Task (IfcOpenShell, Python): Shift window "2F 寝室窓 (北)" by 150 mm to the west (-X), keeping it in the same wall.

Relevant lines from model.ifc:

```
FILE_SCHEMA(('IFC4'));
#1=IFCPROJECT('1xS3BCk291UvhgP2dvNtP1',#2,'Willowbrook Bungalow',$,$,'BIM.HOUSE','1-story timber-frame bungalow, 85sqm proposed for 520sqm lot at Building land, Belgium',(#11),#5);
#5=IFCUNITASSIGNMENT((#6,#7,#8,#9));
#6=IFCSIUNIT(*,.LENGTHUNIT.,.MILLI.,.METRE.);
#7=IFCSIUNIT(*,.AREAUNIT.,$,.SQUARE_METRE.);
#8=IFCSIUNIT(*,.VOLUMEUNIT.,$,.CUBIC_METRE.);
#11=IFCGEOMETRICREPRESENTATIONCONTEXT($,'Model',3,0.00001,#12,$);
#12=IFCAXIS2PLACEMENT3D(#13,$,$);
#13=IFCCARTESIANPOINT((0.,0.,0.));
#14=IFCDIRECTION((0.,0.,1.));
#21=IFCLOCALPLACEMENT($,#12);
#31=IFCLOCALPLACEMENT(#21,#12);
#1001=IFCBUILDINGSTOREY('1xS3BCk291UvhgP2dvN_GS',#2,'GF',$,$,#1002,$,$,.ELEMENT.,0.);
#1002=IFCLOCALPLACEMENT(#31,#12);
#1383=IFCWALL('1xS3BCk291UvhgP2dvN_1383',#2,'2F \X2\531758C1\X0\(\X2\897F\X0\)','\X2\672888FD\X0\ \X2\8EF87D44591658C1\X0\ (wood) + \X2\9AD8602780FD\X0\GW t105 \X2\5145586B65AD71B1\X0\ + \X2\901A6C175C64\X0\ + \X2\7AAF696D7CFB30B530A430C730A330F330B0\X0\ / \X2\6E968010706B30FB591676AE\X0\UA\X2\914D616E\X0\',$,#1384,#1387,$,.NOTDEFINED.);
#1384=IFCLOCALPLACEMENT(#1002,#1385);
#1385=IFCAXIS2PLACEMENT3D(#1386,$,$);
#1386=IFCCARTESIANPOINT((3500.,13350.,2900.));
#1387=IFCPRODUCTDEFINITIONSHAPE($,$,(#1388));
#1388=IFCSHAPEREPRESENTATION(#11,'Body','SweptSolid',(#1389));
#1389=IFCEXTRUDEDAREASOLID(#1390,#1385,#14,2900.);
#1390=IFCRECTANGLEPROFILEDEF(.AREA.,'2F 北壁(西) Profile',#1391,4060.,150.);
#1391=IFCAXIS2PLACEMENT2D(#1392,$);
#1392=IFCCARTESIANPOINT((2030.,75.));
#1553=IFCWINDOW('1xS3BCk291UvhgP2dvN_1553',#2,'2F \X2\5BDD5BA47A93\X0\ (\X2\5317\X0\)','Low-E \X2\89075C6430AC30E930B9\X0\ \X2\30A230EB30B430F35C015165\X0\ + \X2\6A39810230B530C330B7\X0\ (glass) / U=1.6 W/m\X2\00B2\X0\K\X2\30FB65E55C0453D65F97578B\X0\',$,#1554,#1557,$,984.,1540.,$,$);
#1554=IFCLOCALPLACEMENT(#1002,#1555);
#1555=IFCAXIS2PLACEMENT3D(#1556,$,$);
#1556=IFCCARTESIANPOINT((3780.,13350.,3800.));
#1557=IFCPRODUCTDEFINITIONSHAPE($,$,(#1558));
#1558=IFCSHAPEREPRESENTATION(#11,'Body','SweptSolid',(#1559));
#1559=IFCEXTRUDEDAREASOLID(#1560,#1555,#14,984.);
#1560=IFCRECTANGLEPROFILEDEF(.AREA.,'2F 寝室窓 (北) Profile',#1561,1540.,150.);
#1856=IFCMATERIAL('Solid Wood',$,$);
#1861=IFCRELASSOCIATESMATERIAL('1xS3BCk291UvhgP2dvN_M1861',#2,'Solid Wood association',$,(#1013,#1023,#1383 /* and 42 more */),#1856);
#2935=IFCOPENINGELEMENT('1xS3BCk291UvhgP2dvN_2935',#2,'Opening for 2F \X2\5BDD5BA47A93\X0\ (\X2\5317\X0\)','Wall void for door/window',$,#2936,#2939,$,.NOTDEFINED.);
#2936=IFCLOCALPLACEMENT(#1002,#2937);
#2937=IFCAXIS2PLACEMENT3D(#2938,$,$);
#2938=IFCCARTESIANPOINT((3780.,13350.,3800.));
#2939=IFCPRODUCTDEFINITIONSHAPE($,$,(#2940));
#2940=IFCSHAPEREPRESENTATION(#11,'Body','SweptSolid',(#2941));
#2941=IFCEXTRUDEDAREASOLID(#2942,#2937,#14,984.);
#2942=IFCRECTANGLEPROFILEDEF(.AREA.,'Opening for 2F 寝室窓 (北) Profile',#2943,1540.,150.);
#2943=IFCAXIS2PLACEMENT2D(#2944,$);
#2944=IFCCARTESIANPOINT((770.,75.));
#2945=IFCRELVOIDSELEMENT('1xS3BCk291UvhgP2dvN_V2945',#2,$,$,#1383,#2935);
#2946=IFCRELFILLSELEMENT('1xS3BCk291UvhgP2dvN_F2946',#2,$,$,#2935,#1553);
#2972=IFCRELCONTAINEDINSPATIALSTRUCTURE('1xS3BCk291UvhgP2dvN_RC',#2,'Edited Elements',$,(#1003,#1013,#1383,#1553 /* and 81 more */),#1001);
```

```python
import ifcopenshell
import ifcopenshell.api.geometry
import ifcopenshell.util.placement
import ifcopenshell.util.unit

model = ifcopenshell.open("model.ifc")
unit_scale = ifcopenshell.util.unit.calculate_unit_scale(model)

window = model.by_guid("1xS3BCk291UvhgP2dvN_1553")
opening = window.FillsVoids[0].RelatingOpeningElement
wall = opening.VoidsElements[0].RelatingBuildingElement

wall_matrix = ifcopenshell.util.placement.get_local_placement(wall.ObjectPlacement)
shift = wall_matrix[:3, 0] * -0.15 / unit_scale
before = ifcopenshell.util.placement.get_local_placement(window.ObjectPlacement)[:3, 3].copy()

# The window is not placed relative to its opening, so move both.
for product in (opening, window):
    matrix = ifcopenshell.util.placement.get_local_placement(product.ObjectPlacement)
    matrix[:3, 3] += shift
    ifcopenshell.api.geometry.edit_object_placement(model, product=product, matrix=matrix, is_si=False)

after = ifcopenshell.util.placement.get_local_placement(window.ObjectPlacement)[:3, 3]
print("window moved by", (after - before).round(3) + 0.0)

model.write("model-out.ifc")
```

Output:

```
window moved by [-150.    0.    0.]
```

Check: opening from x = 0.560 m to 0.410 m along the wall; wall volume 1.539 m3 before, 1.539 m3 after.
